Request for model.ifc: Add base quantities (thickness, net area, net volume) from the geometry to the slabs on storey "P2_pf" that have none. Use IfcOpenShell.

First a look at what the model holds.

```python
import ifcopenshell
import ifcopenshell.util.element
import ifcopenshell.util.unit

model = ifcopenshell.open("model.ifc")
print(model.schema)
for unit_type in ("LENGTHUNIT", "AREAUNIT", "VOLUMEUNIT"):
    print(unit_type, ifcopenshell.util.unit.calculate_unit_scale(model, unit_type))
storey = next(s for s in model.by_type("IfcBuildingStorey") if s.Name == "P2_pf")
slabs = [e for e in ifcopenshell.util.element.get_decomposition(storey) if e.is_a("IfcSlab")]
for e in sorted(slabs, key=lambda e: e.id()):
    print(e.id(), e.is_a(), e.Name, list(ifcopenshell.util.element.get_psets(e, qtos_only=True)), sep=" | ")
```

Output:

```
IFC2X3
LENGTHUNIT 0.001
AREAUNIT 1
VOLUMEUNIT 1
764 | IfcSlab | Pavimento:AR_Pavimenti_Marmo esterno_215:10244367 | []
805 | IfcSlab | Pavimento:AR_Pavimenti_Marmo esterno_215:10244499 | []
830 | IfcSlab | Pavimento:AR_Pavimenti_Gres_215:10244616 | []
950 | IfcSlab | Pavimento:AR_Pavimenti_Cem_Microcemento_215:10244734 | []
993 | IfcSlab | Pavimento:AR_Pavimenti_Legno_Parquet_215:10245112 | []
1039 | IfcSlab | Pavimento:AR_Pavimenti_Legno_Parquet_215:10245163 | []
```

```python
import ifcopenshell
import ifcopenshell.api.pset
import ifcopenshell.geom
import ifcopenshell.util.element
import ifcopenshell.util.shape
import ifcopenshell.util.unit

model = ifcopenshell.open("model.ifc")
unit_scale = ifcopenshell.util.unit.calculate_unit_scale(model)
area_scale = ifcopenshell.util.unit.calculate_unit_scale(model, "AREAUNIT")
volume_scale = ifcopenshell.util.unit.calculate_unit_scale(model, "VOLUMEUNIT")
settings = ifcopenshell.geom.settings()

storey = next(s for s in model.by_type("IfcBuildingStorey") if s.Name == "P2_pf")
slabs = [e for e in ifcopenshell.util.element.get_decomposition(storey) if e.is_a("IfcSlab")]

for e in sorted(slabs, key=lambda e: e.id()):
    if ifcopenshell.util.element.get_psets(e, qtos_only=True, should_inherit=False):
        continue
    # Geometry comes back in metres, in the element's own axes.
    shape = ifcopenshell.geom.create_shape(settings, e)
    values = {
        "Width": ifcopenshell.util.shape.get_z(shape.geometry) / unit_scale,
        "NetArea": ifcopenshell.util.shape.get_footprint_area(shape.geometry) / area_scale,
        "NetVolume": ifcopenshell.util.shape.get_volume(shape.geometry) / volume_scale,
    }
    qto = ifcopenshell.api.pset.add_qto(model, product=e, name="BaseQuantities")
    ifcopenshell.api.pset.edit_qto(model, qto=qto, properties=values)
    print(e.id(), {k: round(v, 3) for k, v in values.items()})

model.write("model_edited.ifc")
```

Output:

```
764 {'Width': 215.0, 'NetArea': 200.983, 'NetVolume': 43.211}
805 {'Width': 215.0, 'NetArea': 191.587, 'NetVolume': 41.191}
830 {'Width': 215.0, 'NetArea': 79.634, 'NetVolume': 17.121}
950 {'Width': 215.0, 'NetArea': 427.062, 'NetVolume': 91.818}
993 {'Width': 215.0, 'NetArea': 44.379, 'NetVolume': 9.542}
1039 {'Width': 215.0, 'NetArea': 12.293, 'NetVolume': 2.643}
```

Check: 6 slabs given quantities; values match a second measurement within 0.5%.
